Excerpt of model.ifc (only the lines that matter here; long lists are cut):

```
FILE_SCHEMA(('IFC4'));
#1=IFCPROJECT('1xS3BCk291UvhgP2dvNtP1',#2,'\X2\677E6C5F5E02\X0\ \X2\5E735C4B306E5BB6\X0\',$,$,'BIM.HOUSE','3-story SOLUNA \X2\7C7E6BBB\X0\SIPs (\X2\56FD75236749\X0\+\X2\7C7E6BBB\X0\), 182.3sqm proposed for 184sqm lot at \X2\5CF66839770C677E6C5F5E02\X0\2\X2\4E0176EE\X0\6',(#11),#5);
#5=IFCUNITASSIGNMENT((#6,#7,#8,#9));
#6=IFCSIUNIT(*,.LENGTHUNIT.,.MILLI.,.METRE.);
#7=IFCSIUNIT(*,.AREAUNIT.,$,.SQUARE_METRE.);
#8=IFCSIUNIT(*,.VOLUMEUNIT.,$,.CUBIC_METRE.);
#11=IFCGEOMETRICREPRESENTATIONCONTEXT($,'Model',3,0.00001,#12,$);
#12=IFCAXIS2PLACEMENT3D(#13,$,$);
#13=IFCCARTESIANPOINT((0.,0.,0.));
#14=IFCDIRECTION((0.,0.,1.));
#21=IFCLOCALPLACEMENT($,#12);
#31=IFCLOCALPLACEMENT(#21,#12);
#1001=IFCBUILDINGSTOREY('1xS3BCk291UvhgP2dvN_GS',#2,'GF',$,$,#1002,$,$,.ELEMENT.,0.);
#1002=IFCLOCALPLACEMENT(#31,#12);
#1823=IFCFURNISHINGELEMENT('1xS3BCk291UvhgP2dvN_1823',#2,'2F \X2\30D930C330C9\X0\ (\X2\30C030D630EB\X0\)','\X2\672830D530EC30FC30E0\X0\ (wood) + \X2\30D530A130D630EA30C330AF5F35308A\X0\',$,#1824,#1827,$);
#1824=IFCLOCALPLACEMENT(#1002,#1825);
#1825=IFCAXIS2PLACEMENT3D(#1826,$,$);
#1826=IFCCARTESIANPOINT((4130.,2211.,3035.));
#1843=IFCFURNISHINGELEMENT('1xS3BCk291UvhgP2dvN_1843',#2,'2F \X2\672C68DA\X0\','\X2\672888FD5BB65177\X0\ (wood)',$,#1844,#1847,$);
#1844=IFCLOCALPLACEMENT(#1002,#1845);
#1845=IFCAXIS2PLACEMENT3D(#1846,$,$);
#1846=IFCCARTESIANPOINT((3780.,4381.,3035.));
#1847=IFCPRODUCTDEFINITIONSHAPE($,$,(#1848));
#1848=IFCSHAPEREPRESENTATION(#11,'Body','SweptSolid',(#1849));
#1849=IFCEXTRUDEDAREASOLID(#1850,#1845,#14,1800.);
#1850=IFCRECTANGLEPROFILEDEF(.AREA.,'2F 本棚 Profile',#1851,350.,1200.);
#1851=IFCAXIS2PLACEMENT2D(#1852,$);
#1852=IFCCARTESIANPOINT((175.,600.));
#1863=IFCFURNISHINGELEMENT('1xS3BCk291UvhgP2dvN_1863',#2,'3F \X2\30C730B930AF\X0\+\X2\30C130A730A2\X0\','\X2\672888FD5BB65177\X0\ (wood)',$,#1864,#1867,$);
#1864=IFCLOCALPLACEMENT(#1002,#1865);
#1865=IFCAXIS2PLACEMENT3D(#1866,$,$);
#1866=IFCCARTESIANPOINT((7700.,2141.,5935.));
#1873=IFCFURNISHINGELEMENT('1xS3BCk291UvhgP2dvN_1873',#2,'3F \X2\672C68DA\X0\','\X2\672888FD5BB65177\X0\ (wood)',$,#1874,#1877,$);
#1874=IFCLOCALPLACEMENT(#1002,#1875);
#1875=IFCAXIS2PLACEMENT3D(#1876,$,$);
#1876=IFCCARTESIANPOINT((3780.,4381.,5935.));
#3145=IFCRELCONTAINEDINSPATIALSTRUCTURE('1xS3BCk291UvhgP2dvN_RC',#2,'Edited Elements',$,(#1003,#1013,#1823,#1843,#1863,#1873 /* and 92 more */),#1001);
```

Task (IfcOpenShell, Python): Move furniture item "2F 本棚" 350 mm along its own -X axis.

```python
import ifcopenshell
import ifcopenshell.api.geometry
import ifcopenshell.util.placement
import ifcopenshell.util.unit

model = ifcopenshell.open("model.ifc")
unit_scale = ifcopenshell.util.unit.calculate_unit_scale(model)

item = model.by_guid("1xS3BCk291UvhgP2dvN_1843")
matrix = ifcopenshell.util.placement.get_local_placement(item.ObjectPlacement)
matrix[:3, 3] -= matrix[:3, 0] * 0.35 / unit_scale
ifcopenshell.api.geometry.edit_object_placement(model, product=item, matrix=matrix, is_si=False)

print(ifcopenshell.util.placement.get_local_placement(item.ObjectPlacement).round(3) + 0.0)

model.write("model_v2.ifc")
```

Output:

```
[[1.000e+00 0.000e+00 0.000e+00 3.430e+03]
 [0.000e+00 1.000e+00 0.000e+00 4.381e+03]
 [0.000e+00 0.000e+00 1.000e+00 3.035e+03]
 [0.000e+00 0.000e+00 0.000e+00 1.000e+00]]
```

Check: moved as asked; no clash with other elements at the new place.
